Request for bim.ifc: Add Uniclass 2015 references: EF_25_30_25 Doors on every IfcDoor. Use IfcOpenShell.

First a look at what the model holds.

```python
import ifcopenshell

model = ifcopenshell.open("bim.ifc")
print(model.schema)
print("classifications:", [c.Name for c in model.by_type("IfcClassification")])
for ifc_class in ("IfcDoor", "IfcRoof", "IfcStair", "IfcWall", "IfcWindow"):
    print(ifc_class, len(model.by_type(ifc_class)))
```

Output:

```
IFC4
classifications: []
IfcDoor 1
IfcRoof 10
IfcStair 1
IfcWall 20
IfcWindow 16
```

```python
import ifcopenshell
import ifcopenshell.api.classification

model = ifcopenshell.open("bim.ifc")

system = ifcopenshell.api.classification.add_classification(model, classification="Uniclass 2015")

codes = {
    "IfcDoor": ("EF_25_30_25", "Doors"),
}
for ifc_class, (code, name) in codes.items():
    products = model.by_type(ifc_class)
    ifcopenshell.api.classification.add_reference(
        model, products=products, classification=system, identification=code, name=name
    )
    print(code, len(products))

model.write("bim_updated.ifc")
```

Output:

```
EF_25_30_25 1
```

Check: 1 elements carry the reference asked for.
